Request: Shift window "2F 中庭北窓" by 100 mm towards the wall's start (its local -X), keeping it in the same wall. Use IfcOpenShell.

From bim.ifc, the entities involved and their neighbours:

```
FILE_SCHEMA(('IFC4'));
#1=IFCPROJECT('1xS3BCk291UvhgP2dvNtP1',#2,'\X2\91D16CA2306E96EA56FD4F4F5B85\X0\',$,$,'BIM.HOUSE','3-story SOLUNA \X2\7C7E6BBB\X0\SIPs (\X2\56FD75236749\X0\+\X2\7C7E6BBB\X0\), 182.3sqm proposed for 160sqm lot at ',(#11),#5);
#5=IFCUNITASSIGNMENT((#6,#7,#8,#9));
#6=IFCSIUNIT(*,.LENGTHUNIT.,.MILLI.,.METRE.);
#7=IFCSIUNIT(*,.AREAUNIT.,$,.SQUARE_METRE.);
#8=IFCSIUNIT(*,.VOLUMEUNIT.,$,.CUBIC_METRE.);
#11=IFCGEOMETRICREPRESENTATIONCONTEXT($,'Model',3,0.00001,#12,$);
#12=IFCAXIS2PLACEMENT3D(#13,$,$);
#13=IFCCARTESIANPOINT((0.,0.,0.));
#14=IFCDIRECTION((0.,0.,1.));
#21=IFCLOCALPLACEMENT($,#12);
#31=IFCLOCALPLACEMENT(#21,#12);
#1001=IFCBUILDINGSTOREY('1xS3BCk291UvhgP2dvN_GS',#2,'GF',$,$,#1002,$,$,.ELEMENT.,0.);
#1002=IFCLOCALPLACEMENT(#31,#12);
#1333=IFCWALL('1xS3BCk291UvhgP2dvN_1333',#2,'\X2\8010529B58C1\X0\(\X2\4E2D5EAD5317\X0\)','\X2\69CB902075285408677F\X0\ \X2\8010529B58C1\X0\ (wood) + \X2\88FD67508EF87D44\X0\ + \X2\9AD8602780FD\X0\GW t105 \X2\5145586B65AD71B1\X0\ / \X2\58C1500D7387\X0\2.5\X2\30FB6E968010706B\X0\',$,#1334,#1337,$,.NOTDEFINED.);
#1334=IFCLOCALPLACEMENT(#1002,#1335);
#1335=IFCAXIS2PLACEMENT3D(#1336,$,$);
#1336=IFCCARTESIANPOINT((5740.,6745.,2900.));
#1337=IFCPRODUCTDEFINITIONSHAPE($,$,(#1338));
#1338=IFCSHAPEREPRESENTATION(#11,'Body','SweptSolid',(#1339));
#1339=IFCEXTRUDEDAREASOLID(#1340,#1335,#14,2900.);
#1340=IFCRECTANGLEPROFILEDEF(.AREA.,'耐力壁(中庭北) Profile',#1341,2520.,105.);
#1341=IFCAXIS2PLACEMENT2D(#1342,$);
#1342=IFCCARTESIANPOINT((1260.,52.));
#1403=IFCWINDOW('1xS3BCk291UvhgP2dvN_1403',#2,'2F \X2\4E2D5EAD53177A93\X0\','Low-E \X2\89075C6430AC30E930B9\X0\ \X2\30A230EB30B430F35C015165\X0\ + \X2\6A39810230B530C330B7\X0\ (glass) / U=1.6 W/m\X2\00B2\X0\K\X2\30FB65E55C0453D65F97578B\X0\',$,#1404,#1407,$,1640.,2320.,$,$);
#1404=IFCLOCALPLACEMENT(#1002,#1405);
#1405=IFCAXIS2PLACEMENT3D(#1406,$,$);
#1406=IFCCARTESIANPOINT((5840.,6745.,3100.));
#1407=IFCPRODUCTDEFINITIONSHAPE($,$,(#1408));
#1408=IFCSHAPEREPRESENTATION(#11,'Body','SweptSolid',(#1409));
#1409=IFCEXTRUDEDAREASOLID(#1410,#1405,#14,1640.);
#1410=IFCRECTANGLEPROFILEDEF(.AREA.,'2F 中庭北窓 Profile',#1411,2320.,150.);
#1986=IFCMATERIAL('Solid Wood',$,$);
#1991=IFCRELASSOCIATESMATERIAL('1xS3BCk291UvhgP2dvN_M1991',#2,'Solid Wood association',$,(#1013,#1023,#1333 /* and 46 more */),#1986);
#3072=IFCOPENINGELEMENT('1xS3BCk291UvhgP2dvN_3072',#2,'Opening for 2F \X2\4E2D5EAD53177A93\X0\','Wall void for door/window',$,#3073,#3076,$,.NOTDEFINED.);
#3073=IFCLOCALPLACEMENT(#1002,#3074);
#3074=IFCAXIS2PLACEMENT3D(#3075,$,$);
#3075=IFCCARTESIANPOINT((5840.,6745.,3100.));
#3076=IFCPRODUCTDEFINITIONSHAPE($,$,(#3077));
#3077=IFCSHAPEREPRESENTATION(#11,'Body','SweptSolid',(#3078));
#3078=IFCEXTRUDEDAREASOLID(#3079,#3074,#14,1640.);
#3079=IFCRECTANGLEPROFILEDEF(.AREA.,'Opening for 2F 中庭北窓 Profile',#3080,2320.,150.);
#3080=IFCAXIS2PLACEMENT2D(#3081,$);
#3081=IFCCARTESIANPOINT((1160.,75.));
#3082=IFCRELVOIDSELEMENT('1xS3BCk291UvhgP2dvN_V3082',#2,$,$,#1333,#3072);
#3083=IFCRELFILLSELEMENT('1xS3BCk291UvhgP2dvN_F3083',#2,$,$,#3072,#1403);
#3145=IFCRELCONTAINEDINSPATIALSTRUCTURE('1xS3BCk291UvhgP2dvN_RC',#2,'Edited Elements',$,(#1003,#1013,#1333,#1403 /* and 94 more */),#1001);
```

```python
import ifcopenshell
import ifcopenshell.api.geometry
import ifcopenshell.util.placement

model = ifcopenshell.open("bim.ifc")

window = model.by_guid("1xS3BCk291UvhgP2dvN_1403")
opening = window.FillsVoids[0].RelatingOpeningElement
wall = opening.VoidsElements[0].RelatingBuildingElement

wall_matrix = ifcopenshell.util.placement.get_local_placement(wall.ObjectPlacement)
shift = wall_matrix[:3, 0] * -100.0
before = ifcopenshell.util.placement.get_local_placement(window.ObjectPlacement)[:3, 3].copy()

# The window is not placed relative to its opening, so move both.
for product in (opening, window):
    matrix = ifcopenshell.util.placement.get_local_placement(product.ObjectPlacement)
    matrix[:3, 3] += shift
    ifcopenshell.api.geometry.edit_object_placement(model, product=product, matrix=matrix, is_si=False)

after = ifcopenshell.util.placement.get_local_placement(window.ObjectPlacement)[:3, 3]
print("window moved by", (after - before).round(3) + 0.0)

model.write("bim_rev.ifc")
```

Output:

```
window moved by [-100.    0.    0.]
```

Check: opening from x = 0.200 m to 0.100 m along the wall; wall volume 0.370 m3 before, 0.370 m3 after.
